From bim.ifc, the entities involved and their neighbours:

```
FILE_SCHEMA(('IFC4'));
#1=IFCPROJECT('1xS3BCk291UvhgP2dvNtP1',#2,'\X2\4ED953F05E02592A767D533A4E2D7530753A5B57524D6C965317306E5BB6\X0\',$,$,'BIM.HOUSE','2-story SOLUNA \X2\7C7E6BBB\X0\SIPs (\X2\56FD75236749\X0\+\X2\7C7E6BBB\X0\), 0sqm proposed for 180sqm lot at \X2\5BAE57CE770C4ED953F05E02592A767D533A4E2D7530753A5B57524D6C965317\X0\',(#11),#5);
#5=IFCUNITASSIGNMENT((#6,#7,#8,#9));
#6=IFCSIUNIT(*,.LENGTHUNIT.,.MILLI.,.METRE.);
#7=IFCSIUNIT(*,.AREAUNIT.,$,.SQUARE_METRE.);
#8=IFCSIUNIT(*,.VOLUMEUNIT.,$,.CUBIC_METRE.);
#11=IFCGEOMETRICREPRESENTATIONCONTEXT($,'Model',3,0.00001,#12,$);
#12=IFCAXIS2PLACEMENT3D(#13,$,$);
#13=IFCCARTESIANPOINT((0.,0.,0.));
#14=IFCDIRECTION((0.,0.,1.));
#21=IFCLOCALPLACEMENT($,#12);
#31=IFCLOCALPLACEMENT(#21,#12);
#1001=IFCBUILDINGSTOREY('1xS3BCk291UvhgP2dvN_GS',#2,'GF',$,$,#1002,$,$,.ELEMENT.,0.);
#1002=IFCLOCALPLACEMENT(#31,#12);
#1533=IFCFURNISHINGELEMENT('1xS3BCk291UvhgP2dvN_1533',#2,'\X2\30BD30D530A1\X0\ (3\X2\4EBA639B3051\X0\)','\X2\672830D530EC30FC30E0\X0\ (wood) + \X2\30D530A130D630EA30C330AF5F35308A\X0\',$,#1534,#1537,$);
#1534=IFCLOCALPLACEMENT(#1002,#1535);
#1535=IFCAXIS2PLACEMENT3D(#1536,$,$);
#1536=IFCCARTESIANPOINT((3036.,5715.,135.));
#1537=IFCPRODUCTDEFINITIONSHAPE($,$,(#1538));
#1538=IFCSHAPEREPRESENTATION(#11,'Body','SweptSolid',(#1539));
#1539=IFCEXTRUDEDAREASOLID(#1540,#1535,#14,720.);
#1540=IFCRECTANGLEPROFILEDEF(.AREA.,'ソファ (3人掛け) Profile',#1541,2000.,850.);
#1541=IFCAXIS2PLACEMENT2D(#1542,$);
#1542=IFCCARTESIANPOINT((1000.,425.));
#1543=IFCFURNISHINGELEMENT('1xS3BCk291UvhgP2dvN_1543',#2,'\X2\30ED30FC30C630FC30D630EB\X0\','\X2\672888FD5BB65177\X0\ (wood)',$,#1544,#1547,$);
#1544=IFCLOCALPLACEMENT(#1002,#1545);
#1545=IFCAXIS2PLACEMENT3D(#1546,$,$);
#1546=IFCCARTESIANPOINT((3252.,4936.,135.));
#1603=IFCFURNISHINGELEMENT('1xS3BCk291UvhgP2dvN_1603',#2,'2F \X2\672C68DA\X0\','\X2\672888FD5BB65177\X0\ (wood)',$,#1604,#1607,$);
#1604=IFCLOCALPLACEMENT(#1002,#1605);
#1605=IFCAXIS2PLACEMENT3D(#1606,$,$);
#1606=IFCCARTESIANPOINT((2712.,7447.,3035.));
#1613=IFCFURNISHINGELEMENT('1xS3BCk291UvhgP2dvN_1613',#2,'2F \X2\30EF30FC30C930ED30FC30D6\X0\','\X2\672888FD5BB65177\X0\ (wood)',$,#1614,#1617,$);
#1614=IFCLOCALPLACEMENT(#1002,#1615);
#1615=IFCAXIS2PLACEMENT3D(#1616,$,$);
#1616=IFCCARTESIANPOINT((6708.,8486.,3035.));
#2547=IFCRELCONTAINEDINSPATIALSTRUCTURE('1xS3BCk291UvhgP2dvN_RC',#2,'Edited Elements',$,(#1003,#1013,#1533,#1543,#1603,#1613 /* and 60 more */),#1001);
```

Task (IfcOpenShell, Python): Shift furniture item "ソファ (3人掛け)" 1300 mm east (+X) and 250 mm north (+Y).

```python
import ifcopenshell
import ifcopenshell.api.geometry
import ifcopenshell.util.placement
import ifcopenshell.util.unit

model = ifcopenshell.open("bim.ifc")
unit_scale = ifcopenshell.util.unit.calculate_unit_scale(model)

item = model.by_guid("1xS3BCk291UvhgP2dvN_1533")
matrix = ifcopenshell.util.placement.get_local_placement(item.ObjectPlacement)
matrix[0, 3] += 1.3 / unit_scale
matrix[1, 3] += 0.25 / unit_scale
ifcopenshell.api.geometry.edit_object_placement(model, product=item, matrix=matrix, is_si=False)

print(ifcopenshell.util.placement.get_local_placement(item.ObjectPlacement).round(3) + 0.0)

model.write("bim_updated.ifc")
```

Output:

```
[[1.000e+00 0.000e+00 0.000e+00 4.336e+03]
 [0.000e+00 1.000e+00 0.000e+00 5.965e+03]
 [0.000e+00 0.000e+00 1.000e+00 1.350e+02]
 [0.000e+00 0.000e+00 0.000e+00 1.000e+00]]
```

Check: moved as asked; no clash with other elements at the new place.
